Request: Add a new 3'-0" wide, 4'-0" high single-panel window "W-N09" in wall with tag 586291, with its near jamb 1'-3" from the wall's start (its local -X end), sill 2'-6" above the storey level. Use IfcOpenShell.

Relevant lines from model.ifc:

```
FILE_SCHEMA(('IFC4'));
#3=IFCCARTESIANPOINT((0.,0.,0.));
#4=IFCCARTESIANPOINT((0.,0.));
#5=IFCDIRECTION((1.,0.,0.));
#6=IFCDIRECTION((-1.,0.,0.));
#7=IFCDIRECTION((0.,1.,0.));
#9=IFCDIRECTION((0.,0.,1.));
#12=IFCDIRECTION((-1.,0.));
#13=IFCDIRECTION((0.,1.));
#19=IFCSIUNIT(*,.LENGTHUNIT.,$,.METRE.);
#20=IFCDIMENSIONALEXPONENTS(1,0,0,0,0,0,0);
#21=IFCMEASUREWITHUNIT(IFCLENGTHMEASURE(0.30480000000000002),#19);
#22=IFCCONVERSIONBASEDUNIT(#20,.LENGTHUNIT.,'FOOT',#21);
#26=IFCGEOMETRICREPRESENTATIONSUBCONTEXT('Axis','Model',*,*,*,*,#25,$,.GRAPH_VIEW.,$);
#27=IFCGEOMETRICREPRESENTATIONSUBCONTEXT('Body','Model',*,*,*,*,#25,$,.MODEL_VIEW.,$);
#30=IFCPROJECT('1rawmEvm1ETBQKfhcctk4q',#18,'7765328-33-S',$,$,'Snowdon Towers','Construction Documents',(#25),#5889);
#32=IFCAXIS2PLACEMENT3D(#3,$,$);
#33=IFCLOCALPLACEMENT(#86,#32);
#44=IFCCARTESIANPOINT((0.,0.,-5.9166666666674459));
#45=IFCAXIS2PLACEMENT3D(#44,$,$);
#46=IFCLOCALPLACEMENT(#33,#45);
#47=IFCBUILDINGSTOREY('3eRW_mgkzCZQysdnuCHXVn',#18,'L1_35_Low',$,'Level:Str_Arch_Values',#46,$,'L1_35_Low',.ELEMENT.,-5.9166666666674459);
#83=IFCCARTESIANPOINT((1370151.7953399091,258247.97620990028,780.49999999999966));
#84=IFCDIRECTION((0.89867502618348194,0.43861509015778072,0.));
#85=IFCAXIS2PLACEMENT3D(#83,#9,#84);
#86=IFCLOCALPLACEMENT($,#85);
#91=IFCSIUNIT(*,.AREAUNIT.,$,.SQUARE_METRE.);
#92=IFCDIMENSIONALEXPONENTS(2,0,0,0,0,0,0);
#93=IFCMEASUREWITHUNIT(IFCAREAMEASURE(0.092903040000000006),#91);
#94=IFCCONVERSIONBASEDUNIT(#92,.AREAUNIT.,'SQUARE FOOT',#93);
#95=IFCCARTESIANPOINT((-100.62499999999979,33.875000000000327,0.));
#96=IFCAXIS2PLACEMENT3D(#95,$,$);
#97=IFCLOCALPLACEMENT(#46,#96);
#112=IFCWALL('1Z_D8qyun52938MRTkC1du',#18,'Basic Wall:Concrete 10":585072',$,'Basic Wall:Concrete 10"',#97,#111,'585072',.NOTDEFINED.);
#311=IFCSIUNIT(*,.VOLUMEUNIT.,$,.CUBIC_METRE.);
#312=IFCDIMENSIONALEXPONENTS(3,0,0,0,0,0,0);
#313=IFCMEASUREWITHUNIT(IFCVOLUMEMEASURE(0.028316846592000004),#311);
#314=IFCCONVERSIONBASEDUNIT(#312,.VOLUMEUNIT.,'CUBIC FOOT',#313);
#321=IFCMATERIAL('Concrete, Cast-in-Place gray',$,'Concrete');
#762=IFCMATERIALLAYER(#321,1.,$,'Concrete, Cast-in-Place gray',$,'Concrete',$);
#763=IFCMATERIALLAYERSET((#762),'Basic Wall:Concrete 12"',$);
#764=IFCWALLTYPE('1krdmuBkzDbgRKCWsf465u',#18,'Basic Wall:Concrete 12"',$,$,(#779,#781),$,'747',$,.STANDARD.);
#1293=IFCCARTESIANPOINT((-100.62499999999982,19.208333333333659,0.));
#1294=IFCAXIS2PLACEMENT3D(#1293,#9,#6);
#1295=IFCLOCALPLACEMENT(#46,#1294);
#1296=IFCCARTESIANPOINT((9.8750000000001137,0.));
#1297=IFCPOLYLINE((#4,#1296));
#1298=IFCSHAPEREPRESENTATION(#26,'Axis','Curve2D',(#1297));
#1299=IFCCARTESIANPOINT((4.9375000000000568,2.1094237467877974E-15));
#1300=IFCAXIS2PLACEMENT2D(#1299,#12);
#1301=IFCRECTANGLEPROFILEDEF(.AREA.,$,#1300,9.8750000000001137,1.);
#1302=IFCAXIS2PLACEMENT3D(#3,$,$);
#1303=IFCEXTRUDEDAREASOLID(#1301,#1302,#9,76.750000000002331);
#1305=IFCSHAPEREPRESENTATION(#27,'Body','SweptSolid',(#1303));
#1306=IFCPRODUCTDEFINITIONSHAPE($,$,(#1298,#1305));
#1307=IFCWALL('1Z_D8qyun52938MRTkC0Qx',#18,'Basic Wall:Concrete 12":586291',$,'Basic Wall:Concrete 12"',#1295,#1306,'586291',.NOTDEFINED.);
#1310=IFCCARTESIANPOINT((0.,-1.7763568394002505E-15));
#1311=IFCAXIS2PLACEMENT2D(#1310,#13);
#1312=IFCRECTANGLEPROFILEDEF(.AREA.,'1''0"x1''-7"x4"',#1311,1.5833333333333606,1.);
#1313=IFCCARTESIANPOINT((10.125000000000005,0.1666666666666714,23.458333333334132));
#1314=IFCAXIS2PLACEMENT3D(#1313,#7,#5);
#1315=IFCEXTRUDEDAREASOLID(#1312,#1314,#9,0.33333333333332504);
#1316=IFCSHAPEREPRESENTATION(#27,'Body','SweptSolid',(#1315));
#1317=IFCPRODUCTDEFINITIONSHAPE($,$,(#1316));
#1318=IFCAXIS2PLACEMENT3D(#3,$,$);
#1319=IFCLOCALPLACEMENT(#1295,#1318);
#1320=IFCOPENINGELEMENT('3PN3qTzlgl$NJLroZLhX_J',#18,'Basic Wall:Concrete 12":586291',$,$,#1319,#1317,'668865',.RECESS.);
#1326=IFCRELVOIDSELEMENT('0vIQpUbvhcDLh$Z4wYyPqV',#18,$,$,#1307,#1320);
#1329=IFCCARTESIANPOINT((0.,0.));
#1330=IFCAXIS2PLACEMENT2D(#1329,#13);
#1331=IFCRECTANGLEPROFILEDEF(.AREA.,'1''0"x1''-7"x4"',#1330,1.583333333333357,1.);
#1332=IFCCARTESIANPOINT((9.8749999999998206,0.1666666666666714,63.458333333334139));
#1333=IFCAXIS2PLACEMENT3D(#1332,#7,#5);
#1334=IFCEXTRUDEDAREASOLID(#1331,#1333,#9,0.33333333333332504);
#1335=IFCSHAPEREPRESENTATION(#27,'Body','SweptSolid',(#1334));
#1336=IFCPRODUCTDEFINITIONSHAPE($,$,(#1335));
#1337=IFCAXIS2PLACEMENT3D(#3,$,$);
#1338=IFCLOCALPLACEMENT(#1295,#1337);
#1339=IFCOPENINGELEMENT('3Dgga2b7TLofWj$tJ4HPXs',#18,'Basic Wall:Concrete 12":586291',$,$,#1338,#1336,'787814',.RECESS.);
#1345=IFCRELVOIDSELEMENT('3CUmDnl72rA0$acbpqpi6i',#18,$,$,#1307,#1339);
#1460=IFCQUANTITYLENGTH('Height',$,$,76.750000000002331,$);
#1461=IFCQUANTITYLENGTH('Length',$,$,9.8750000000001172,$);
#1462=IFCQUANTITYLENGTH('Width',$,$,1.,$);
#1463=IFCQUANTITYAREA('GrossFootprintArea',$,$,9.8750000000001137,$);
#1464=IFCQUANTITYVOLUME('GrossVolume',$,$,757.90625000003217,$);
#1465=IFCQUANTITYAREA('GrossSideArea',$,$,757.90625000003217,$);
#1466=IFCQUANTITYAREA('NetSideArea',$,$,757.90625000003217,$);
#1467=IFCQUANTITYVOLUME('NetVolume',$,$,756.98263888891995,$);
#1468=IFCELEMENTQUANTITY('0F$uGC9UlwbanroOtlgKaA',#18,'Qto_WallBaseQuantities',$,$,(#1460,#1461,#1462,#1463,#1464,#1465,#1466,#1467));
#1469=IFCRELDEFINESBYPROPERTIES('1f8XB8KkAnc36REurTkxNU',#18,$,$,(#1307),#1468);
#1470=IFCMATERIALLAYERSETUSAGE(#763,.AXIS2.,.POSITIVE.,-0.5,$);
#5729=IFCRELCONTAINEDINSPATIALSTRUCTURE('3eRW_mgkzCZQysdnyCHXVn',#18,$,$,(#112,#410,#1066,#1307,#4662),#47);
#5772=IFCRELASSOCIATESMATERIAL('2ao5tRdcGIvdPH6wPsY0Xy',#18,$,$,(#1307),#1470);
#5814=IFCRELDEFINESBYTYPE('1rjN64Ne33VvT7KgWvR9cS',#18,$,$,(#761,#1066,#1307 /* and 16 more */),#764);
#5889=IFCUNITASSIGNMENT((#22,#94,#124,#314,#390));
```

```python
import numpy as np
import ifcopenshell
import ifcopenshell.api.feature
import ifcopenshell.api.geometry
import ifcopenshell.api.pset
import ifcopenshell.api.root
import ifcopenshell.api.spatial
import ifcopenshell.geom
import ifcopenshell.util.element
import ifcopenshell.util.placement
import ifcopenshell.util.representation
import ifcopenshell.util.shape
import ifcopenshell.util.unit

model = ifcopenshell.open("model.ifc")
unit_scale = ifcopenshell.util.unit.calculate_unit_scale(model)
area_scale = ifcopenshell.util.unit.calculate_unit_scale(model, "AREAUNIT")
volume_scale = ifcopenshell.util.unit.calculate_unit_scale(model, "VOLUMEUNIT")
settings = ifcopenshell.geom.settings()


def volume(element):
    """Net volume in cubic metres, openings subtracted."""
    shape = ifcopenshell.geom.create_shape(settings, element)
    return ifcopenshell.util.shape.get_volume(shape.geometry)


wall = model.by_guid("1Z_D8qyun52938MRTkC0Qx")
storey = ifcopenshell.util.element.get_container(wall, ifc_class="IfcBuildingStorey")
context = ifcopenshell.util.representation.get_context(model, "Model", "Body", "MODEL_VIEW")
before = volume(wall)

width, height, from_end, sill = 0.9144, 1.2192, 0.381, 0.762  # metres

# The wall runs along its own X axis, and the end named is its -X end.
wall_shape = ifcopenshell.geom.create_shape(settings, wall)
x, y, z = ifcopenshell.util.shape.get_vertices(wall_shape.geometry).T
start = x.min() + from_end
face, thickness = float(y.min()), float(y.max() - y.min())
wall_matrix = ifcopenshell.util.placement.get_local_placement(wall.ObjectPlacement)
level = ifcopenshell.util.placement.get_local_placement(storey.ObjectPlacement)[2, 3]


def in_wall(x, y):
    """Placement at x, y metres in the wall's axes, at sill height."""
    matrix = wall_matrix.copy()
    matrix[:, 3] = wall_matrix @ np.array([x / unit_scale, y / unit_scale, 0.0, 1.0])
    matrix[2, 3] = level + sill / unit_scale
    return matrix


# Opening: a box that overshoots both wall faces by 50 mm.
opening = ifcopenshell.api.root.create_entity(model, ifc_class="IfcOpeningElement", predefined_type="OPENING")
box = ifcopenshell.api.geometry.add_wall_representation(
    model, context=context, length=width, height=height, thickness=thickness + 0.1
)
ifcopenshell.api.geometry.assign_representation(model, product=opening, representation=box)
ifcopenshell.api.geometry.edit_object_placement(model, product=opening, matrix=in_wall(start, face - 0.05), is_si=False)
ifcopenshell.api.feature.add_feature(model, feature=opening, element=wall)

window = ifcopenshell.api.root.create_entity(model, ifc_class="IfcWindow", name="W-N09", predefined_type="WINDOW")
window.OverallWidth, window.OverallHeight = width / unit_scale, height / unit_scale
window.PartitioningType = "SINGLE_PANEL"
body = ifcopenshell.api.geometry.add_window_representation(
    model,
    context=context,
    overall_width=window.OverallWidth,
    overall_height=window.OverallHeight,
    partition_type="SINGLE_PANEL",
)
ifcopenshell.api.geometry.assign_representation(model, product=window, representation=body)
ifcopenshell.api.spatial.assign_container(model, products=[window], relating_structure=storey)
ifcopenshell.api.feature.add_filling(model, opening=opening, element=window)

# Centre the window in the wall's thickness.
ifcopenshell.api.geometry.edit_object_placement(model, product=window, matrix=in_wall(start, face), is_si=False)
window_shape = ifcopenshell.geom.create_shape(settings, window)
depth = ifcopenshell.util.shape.get_vertices(window_shape.geometry)[:, 1]
offset = face + thickness / 2 - (depth.min() + depth.max()) / 2
ifcopenshell.api.geometry.edit_object_placement(model, product=window, matrix=in_wall(start, offset), is_si=False)

after = volume(wall)

# Update the wall's stored quantities.
qto = model.by_id(ifcopenshell.util.element.get_pset(wall, "Qto_WallBaseQuantities", should_inherit=False)["id"])
ifcopenshell.api.pset.edit_qto(model, qto=qto, properties={
    "NetSideArea": after / thickness / area_scale,
    "NetVolume": after / volume_scale,
})

print(f"wall volume {before:.3f} -> {after:.3f} m3")

model.write("model-out.ifc")
```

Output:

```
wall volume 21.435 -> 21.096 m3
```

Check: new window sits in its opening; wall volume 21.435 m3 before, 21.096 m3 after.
